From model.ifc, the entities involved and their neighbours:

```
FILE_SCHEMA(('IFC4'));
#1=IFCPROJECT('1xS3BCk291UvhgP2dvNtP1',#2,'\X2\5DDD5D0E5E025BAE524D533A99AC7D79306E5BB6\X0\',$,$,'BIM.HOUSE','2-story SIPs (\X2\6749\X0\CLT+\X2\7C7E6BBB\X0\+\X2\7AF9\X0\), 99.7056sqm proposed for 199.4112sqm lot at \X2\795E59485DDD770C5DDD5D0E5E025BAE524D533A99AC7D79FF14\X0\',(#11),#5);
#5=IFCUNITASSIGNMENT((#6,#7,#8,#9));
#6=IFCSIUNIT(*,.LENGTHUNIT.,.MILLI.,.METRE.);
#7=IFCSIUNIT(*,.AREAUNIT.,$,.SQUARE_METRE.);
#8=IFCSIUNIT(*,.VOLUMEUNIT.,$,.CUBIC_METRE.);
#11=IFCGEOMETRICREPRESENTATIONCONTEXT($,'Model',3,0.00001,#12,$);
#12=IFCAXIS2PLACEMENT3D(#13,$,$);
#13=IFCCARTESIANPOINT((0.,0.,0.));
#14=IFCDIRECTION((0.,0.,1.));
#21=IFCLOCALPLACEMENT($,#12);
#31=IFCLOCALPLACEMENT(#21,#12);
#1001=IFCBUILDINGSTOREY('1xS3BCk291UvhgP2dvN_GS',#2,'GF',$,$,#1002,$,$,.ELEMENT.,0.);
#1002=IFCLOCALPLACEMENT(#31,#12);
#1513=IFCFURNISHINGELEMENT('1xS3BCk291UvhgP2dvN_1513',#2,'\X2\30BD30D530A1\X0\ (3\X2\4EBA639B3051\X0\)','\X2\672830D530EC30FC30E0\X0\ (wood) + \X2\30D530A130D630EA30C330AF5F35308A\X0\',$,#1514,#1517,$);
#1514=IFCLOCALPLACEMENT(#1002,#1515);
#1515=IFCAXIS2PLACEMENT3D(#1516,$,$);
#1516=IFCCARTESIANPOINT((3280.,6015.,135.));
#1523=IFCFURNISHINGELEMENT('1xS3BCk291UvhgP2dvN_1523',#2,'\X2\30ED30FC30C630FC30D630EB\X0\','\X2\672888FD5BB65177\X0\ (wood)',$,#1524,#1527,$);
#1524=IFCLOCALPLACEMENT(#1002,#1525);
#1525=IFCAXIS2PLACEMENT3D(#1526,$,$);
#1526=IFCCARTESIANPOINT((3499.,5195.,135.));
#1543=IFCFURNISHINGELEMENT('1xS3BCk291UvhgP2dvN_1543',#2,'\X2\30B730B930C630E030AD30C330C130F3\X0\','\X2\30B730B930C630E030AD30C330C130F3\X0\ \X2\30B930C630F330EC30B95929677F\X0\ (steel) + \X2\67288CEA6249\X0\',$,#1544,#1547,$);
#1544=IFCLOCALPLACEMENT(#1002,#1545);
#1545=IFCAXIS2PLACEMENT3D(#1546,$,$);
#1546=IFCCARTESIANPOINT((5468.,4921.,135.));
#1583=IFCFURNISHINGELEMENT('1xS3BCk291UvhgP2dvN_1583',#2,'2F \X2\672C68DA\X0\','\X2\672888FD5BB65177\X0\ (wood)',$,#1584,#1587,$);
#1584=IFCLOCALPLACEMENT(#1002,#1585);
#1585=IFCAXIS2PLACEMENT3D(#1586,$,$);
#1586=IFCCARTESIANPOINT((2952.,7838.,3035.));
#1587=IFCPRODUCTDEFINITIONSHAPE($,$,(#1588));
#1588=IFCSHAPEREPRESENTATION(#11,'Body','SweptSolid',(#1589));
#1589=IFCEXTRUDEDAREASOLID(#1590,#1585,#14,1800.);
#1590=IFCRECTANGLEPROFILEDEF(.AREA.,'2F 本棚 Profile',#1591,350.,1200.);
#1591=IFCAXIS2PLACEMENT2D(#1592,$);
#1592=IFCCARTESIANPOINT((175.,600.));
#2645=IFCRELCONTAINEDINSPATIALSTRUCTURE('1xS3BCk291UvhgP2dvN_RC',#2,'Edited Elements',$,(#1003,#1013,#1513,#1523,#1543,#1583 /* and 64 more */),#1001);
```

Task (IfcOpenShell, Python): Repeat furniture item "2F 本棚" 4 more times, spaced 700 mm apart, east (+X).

```python
import numpy as np
import ifcopenshell
import ifcopenshell.api.geometry
import ifcopenshell.api.root
import ifcopenshell.util.element
import ifcopenshell.util.placement
import ifcopenshell.util.unit

model = ifcopenshell.open("model.ifc")
unit_scale = ifcopenshell.util.unit.calculate_unit_scale(model)


def reuse_history(source, copy):
    """copy_class also copies each property set's owner history, people and application; keep the originals."""
    for rel in copy.IsDefinedBy:
        if rel.is_a("IfcRelDefinesByProperties") and (history := rel.RelatingPropertyDefinition.OwnerHistory):
            rel.RelatingPropertyDefinition.OwnerHistory = source.OwnerHistory
            ifcopenshell.util.element.remove_deep2(model, history)


source = model.by_guid("1xS3BCk291UvhgP2dvN_1583")
base = ifcopenshell.util.placement.get_local_placement(source.ObjectPlacement)
step = np.array([1.0, 0.0, 0.0]) * 0.7 / unit_scale

for i in range(1, 5):
    copy = ifcopenshell.api.root.copy_class(model, product=source)
    copy.Representation = ifcopenshell.util.element.copy_deep(
        model, source.Representation, exclude=["IfcGeometricRepresentationContext", "IfcRepresentationMap"]
    )
    reuse_history(source, copy)
    matrix = base.copy()
    matrix[:3, 3] += i * step
    print("added at", matrix[:3, 3].round(3) + 0.0)
    ifcopenshell.api.geometry.edit_object_placement(model, product=copy, matrix=matrix, is_si=False)

model.write("model_edited.ifc")
```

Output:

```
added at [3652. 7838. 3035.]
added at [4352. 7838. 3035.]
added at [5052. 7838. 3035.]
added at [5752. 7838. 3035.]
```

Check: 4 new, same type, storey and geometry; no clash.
